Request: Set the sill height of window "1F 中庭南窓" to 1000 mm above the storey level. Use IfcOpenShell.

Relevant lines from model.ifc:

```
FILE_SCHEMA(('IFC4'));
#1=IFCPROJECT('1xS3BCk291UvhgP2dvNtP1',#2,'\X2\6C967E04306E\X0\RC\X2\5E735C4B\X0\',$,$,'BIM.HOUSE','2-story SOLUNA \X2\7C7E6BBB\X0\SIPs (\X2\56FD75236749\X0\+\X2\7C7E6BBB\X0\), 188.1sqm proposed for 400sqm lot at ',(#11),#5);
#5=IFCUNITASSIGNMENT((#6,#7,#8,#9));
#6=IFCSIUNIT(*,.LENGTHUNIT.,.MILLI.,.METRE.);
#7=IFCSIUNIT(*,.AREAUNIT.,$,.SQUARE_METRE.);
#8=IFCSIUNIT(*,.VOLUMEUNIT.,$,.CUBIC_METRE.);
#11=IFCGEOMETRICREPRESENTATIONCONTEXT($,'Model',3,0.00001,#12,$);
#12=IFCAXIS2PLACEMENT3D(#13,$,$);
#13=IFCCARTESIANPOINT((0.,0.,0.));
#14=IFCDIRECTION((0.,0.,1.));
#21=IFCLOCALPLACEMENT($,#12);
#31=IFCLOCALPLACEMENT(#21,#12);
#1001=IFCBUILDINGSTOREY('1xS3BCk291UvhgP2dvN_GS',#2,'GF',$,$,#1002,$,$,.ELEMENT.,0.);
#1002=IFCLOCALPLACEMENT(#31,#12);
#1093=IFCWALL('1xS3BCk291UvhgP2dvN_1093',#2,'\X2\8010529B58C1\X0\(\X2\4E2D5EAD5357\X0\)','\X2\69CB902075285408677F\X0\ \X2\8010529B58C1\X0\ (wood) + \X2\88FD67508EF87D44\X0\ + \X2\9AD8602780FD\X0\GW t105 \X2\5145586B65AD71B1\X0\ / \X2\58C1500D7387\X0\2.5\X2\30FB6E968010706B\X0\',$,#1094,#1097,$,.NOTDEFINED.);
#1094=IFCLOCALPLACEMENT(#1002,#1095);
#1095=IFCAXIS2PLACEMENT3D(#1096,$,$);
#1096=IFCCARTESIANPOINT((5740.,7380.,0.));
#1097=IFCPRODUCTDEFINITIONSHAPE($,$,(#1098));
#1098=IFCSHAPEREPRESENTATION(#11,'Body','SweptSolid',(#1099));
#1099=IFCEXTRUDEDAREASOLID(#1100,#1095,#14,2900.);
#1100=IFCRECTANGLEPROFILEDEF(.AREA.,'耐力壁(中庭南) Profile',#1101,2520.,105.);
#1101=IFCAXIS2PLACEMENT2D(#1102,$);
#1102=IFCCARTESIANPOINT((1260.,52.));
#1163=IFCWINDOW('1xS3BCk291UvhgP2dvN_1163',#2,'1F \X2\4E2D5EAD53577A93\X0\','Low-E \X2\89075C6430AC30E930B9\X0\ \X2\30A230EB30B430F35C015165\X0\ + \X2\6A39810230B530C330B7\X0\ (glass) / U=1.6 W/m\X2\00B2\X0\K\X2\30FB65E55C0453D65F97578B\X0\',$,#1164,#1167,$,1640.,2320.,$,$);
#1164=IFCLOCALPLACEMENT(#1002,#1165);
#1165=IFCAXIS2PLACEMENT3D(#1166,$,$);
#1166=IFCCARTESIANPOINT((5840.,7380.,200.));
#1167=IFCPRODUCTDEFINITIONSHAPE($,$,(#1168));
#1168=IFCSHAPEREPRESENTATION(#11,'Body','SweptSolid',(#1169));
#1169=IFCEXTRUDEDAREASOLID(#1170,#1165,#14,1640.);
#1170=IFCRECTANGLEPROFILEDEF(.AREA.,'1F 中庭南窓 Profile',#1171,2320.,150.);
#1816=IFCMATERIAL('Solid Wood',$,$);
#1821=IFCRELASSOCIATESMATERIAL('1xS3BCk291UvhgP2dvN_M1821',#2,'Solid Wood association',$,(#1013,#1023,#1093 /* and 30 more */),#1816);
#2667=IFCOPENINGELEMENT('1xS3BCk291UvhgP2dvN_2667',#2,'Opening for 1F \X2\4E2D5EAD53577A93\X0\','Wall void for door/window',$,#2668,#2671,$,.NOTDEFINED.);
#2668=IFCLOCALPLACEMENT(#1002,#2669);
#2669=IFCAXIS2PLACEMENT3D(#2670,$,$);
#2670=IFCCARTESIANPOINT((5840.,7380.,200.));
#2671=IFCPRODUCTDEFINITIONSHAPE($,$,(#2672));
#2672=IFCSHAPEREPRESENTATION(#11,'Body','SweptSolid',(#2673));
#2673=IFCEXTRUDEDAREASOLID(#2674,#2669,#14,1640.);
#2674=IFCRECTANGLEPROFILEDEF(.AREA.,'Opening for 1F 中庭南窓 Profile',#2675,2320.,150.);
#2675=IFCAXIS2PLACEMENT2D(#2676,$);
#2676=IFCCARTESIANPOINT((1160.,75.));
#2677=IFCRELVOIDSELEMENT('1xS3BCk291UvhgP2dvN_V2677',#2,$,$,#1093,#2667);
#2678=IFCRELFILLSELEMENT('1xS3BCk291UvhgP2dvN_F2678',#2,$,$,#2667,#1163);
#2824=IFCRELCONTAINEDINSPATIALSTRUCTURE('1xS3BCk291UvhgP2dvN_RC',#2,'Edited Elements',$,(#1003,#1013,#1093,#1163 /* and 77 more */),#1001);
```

```python
import numpy as np
import ifcopenshell
import ifcopenshell.api.geometry
import ifcopenshell.geom
import ifcopenshell.util.element
import ifcopenshell.util.placement
import ifcopenshell.util.shape
import ifcopenshell.util.unit

model = ifcopenshell.open("model.ifc")
unit_scale = ifcopenshell.util.unit.calculate_unit_scale(model)

window = model.by_id(1163)
opening = window.FillsVoids[0].RelatingOpeningElement
storey = ifcopenshell.util.element.get_container(window, ifc_class="IfcBuildingStorey")
level = ifcopenshell.util.placement.get_local_placement(storey.ObjectPlacement)[2, 3]

# The opening's origin need not be at the sill, so measure its lowest point.
shape = ifcopenshell.geom.create_shape(ifcopenshell.geom.settings(), opening)
bottom = ifcopenshell.util.shape.get_shape_bottom_elevation(shape, shape.geometry) / unit_scale
dz = level + 1000.0 - bottom

shift = np.array([0.0, 0.0, dz])
# The window is not placed relative to its opening, so move both.
for product in (opening, window):
    matrix = ifcopenshell.util.placement.get_local_placement(product.ObjectPlacement)
    matrix[:3, 3] += shift
    ifcopenshell.api.geometry.edit_object_placement(model, product=product, matrix=matrix, is_si=False)

print(f"moved by {dz * unit_scale:+.3f} m")

model.write("model_edited.ifc")
```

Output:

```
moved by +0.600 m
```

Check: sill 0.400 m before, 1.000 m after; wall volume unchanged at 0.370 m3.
